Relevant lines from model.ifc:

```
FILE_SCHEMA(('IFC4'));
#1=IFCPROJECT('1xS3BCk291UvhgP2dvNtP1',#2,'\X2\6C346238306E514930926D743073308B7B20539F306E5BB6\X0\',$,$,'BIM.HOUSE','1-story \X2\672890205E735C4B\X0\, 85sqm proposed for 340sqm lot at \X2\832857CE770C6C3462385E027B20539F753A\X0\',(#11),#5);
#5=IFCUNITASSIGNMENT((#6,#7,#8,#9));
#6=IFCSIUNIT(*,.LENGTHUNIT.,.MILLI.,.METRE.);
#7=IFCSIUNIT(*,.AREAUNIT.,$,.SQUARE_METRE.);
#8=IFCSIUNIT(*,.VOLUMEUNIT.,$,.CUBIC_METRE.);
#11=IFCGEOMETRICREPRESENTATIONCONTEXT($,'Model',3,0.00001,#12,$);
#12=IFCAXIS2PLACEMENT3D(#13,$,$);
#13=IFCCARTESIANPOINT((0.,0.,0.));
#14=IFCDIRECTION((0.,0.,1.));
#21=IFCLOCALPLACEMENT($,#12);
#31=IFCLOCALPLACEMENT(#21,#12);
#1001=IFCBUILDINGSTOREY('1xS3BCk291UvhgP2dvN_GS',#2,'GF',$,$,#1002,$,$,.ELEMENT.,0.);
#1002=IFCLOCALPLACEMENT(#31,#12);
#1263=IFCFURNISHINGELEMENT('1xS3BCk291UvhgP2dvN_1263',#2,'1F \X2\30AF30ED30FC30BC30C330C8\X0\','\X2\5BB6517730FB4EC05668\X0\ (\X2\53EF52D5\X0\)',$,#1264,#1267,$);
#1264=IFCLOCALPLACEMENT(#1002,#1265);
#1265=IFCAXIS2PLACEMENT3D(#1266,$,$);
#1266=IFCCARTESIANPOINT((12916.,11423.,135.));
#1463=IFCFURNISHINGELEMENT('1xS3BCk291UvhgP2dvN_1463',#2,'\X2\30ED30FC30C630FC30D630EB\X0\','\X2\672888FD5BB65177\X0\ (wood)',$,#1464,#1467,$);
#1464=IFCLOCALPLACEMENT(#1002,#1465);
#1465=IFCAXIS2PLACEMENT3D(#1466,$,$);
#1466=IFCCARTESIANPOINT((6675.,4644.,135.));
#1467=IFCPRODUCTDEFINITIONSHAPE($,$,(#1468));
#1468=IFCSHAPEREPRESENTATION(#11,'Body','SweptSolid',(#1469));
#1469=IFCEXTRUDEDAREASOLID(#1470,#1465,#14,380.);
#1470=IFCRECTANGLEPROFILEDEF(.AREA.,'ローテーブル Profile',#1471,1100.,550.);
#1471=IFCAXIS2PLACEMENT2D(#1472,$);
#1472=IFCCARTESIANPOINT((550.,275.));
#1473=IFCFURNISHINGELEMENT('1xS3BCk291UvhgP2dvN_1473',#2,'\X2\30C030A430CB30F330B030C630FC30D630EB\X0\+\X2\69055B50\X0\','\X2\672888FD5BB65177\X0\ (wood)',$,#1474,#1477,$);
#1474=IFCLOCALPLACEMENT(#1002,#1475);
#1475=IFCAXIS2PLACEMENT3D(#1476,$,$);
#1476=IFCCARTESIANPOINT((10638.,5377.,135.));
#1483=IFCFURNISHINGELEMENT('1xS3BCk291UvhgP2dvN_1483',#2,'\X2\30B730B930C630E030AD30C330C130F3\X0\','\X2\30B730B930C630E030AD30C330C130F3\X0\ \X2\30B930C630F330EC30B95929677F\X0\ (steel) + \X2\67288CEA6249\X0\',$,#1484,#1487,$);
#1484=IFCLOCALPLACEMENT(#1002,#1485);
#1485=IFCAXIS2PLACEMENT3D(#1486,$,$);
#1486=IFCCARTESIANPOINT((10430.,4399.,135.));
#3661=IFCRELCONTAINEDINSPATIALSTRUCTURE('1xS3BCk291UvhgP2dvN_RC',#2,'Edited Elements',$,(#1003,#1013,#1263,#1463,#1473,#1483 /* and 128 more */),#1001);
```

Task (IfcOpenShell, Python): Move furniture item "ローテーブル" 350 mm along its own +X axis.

```python
import ifcopenshell
import ifcopenshell.api.geometry
import ifcopenshell.util.placement

model = ifcopenshell.open("model.ifc")

item = model.by_guid("1xS3BCk291UvhgP2dvN_1463")
matrix = ifcopenshell.util.placement.get_local_placement(item.ObjectPlacement)
matrix[:3, 3] += matrix[:3, 0] * 350.0
ifcopenshell.api.geometry.edit_object_placement(model, product=item, matrix=matrix, is_si=False)

print(ifcopenshell.util.placement.get_local_placement(item.ObjectPlacement).round(3) + 0.0)

model.write("model_edited.ifc")
```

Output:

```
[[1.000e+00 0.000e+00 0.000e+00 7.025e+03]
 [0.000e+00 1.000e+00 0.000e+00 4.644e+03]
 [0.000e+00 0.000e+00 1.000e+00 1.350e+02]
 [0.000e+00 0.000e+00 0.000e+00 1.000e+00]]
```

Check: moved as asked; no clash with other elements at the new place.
